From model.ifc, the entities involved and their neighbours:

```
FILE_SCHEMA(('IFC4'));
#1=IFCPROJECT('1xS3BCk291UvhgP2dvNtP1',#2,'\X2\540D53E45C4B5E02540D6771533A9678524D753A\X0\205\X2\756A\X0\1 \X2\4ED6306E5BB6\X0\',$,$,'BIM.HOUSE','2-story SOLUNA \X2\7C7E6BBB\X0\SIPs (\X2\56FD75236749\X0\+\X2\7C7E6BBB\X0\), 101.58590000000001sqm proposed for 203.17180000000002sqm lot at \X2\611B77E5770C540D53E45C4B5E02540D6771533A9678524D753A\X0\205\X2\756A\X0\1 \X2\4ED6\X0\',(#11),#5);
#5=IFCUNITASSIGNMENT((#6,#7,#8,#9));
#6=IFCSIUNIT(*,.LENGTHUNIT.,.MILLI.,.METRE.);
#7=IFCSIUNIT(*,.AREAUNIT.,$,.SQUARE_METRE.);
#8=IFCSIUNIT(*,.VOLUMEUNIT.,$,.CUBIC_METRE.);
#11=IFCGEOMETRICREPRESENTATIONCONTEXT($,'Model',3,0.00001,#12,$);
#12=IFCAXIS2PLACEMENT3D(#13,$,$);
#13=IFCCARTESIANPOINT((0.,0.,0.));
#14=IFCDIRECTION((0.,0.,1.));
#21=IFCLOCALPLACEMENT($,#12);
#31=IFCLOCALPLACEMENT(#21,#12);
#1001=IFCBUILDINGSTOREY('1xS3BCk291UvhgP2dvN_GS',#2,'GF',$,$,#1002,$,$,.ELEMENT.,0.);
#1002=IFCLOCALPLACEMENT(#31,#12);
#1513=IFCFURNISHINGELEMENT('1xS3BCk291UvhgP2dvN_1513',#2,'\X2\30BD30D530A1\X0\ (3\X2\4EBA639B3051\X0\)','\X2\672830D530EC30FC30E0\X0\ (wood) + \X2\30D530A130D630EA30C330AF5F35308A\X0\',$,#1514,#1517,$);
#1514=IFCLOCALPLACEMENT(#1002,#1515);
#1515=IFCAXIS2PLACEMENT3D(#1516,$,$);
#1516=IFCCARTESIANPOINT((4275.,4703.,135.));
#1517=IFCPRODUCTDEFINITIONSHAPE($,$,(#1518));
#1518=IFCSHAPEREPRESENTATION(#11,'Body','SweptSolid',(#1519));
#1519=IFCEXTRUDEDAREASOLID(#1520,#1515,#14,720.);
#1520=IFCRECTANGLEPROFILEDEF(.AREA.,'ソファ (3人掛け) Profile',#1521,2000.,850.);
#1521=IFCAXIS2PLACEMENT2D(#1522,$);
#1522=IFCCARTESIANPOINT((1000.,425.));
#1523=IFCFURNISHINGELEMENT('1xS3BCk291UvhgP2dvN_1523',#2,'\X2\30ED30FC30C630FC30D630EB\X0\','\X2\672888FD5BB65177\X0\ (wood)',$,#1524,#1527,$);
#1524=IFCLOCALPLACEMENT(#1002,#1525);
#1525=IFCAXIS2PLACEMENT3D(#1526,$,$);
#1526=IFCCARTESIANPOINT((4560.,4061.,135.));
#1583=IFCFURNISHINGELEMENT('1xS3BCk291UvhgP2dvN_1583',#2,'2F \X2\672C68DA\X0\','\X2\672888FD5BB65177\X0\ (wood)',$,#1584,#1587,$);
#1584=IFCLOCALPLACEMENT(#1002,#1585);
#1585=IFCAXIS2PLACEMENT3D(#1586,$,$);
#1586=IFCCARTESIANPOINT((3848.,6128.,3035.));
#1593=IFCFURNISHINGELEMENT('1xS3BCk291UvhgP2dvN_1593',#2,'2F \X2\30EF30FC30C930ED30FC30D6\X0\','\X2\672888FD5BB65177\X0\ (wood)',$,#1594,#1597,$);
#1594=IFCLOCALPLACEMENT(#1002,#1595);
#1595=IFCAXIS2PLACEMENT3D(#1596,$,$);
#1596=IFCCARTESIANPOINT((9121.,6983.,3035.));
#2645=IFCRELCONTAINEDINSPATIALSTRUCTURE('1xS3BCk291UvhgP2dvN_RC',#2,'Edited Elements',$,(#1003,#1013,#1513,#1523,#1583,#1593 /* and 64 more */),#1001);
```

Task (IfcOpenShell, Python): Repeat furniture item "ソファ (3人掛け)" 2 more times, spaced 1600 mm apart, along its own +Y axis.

```python
import ifcopenshell
import ifcopenshell.api.geometry
import ifcopenshell.api.root
import ifcopenshell.util.element
import ifcopenshell.util.placement
import ifcopenshell.util.unit

model = ifcopenshell.open("model.ifc")
unit_scale = ifcopenshell.util.unit.calculate_unit_scale(model)


def reuse_history(source, copy):
    """copy_class also copies each property set's owner history, people and application; keep the originals."""
    for rel in copy.IsDefinedBy:
        if rel.is_a("IfcRelDefinesByProperties") and (history := rel.RelatingPropertyDefinition.OwnerHistory):
            rel.RelatingPropertyDefinition.OwnerHistory = source.OwnerHistory
            ifcopenshell.util.element.remove_deep2(model, history)


source = model.by_guid("1xS3BCk291UvhgP2dvN_1513")
base = ifcopenshell.util.placement.get_local_placement(source.ObjectPlacement)
step = base[:3, 1] * 1.6 / unit_scale

for i in range(1, 3):
    copy = ifcopenshell.api.root.copy_class(model, product=source)
    copy.Representation = ifcopenshell.util.element.copy_deep(
        model, source.Representation, exclude=["IfcGeometricRepresentationContext", "IfcRepresentationMap"]
    )
    reuse_history(source, copy)
    matrix = base.copy()
    matrix[:3, 3] += i * step
    print("added at", matrix[:3, 3].round(3) + 0.0)
    ifcopenshell.api.geometry.edit_object_placement(model, product=copy, matrix=matrix, is_si=False)

model.write("model_updated.ifc")
```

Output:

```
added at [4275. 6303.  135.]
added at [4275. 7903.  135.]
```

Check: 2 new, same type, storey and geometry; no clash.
